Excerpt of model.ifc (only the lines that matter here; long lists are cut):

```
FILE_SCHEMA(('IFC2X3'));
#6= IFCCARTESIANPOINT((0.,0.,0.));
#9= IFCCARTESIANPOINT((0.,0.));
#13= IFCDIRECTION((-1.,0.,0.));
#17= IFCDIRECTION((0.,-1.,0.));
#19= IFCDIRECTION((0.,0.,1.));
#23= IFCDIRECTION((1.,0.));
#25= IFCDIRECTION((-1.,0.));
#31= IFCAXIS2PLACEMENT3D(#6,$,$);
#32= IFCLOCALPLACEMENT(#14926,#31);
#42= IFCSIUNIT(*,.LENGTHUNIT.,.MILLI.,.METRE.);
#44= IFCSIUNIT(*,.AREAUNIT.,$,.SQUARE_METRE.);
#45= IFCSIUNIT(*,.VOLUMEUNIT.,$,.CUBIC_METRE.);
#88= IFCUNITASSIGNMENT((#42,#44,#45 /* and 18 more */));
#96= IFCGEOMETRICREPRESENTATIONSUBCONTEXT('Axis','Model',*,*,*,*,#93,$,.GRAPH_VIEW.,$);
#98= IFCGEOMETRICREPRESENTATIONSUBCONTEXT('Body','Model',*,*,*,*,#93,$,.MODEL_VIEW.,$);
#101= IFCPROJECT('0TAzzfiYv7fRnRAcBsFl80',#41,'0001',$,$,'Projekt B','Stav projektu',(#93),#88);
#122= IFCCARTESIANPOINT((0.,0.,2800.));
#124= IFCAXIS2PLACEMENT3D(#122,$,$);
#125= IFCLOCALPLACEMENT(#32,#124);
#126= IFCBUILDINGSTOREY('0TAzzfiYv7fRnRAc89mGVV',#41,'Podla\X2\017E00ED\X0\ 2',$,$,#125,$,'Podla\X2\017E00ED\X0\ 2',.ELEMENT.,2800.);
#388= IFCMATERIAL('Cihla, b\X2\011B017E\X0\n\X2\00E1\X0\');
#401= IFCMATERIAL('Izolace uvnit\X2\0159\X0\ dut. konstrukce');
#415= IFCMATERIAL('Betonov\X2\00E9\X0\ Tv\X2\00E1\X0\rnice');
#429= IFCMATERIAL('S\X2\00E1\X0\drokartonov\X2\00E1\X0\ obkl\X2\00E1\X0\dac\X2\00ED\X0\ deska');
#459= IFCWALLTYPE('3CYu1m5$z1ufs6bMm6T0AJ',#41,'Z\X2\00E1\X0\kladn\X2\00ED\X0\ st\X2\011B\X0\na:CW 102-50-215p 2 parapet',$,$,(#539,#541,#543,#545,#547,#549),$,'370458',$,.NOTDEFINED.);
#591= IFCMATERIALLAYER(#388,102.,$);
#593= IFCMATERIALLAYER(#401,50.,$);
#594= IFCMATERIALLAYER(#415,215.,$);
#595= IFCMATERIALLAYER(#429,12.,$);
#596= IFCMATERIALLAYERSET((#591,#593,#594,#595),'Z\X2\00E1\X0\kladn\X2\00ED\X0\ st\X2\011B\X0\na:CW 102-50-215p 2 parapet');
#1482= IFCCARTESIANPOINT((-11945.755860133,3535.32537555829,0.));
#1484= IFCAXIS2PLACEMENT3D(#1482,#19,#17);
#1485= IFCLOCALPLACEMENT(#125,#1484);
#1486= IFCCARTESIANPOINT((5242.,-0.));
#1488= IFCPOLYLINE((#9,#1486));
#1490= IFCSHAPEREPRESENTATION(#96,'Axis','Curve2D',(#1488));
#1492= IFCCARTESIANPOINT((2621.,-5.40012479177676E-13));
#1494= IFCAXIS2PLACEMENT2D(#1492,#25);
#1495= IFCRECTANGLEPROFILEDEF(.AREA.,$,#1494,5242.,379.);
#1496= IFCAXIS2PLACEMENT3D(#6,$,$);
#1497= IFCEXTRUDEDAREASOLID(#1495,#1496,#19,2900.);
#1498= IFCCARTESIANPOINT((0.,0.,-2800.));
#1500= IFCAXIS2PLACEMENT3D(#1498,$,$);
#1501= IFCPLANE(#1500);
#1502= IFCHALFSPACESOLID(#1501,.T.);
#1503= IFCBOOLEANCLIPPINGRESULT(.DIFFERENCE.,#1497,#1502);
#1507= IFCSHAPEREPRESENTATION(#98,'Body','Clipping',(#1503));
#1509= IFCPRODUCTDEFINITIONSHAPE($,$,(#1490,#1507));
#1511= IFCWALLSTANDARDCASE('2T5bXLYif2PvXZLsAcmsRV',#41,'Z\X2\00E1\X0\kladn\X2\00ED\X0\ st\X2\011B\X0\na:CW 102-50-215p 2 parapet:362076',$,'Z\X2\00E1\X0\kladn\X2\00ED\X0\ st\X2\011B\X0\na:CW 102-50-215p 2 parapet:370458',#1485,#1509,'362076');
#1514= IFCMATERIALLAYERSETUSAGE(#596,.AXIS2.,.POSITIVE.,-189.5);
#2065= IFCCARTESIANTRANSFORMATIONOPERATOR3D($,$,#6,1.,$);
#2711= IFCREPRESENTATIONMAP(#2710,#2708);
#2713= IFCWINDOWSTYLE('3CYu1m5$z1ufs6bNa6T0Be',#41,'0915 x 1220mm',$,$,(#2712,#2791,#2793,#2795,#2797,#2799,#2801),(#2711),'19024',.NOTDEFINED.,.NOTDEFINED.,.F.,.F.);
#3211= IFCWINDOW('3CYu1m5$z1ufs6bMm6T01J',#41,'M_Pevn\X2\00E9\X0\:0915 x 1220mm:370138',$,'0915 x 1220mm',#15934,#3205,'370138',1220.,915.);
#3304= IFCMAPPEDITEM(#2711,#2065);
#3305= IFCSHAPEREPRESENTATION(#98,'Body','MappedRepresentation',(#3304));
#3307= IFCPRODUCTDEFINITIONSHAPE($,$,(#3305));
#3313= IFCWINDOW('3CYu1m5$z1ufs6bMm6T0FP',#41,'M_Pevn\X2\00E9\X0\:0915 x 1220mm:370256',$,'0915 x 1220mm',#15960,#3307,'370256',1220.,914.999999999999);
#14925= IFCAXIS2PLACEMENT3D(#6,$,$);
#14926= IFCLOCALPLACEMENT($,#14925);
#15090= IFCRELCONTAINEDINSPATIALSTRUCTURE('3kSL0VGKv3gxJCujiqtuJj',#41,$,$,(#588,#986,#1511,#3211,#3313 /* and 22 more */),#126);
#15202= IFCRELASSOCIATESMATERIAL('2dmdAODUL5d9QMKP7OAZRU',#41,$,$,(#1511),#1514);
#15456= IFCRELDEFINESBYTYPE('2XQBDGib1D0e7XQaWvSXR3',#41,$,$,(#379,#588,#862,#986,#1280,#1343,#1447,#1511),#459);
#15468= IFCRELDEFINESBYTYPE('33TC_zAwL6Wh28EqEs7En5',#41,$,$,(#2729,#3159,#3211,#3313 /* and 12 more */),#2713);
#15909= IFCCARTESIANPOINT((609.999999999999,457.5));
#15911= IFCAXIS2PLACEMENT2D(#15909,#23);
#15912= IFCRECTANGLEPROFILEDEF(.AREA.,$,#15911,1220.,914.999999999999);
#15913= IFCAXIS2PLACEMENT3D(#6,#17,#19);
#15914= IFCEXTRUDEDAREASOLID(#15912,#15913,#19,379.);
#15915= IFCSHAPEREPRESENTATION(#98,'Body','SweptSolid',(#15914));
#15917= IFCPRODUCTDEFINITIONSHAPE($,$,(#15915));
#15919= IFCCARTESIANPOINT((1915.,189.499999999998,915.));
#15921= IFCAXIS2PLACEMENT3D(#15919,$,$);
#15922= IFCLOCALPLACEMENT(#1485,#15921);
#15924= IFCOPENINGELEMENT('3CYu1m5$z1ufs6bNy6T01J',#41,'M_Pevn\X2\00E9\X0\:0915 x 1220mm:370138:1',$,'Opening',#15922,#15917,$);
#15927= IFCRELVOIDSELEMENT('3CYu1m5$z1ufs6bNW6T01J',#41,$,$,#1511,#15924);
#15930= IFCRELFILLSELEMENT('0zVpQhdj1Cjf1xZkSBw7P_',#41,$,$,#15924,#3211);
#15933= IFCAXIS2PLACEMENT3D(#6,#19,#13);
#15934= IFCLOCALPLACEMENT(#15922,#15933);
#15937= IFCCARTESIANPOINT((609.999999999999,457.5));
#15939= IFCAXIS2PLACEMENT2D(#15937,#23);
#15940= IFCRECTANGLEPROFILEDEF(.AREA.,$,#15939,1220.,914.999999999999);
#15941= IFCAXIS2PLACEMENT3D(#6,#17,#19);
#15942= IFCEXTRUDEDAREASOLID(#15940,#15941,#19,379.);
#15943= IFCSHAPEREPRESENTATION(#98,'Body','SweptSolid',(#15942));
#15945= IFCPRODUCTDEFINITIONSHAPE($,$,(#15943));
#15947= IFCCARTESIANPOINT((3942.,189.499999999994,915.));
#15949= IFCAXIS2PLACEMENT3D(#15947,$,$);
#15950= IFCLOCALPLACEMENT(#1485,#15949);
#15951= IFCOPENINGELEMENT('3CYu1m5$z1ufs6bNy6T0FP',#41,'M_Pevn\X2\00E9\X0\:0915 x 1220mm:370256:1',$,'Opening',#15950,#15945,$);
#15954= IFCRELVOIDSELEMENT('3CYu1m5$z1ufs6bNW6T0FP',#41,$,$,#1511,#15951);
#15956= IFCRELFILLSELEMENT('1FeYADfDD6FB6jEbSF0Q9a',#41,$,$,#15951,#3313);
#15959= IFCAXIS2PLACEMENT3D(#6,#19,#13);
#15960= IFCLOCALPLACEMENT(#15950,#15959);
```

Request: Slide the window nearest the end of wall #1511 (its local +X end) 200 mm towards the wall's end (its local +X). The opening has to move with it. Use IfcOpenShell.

```python
import ifcopenshell
import ifcopenshell.api.geometry
import ifcopenshell.util.placement

model = ifcopenshell.open("model.ifc")

window = model.by_id(3313)
opening = window.FillsVoids[0].RelatingOpeningElement
wall = opening.VoidsElements[0].RelatingBuildingElement

wall_matrix = ifcopenshell.util.placement.get_local_placement(wall.ObjectPlacement)
shift = wall_matrix[:3, 0] * 200.0
before = ifcopenshell.util.placement.get_local_placement(window.ObjectPlacement)[:3, 3].copy()

# The window is placed relative to its opening, so it follows when the opening moves.
matrix = ifcopenshell.util.placement.get_local_placement(opening.ObjectPlacement)
matrix[:3, 3] += shift
ifcopenshell.api.geometry.edit_object_placement(
    model, product=opening, matrix=matrix, is_si=False, should_transform_children=True
)

after = ifcopenshell.util.placement.get_local_placement(window.ObjectPlacement)[:3, 3]
print("window moved by", (after - before).round(3) + 0.0)

model.write("model-out.ifc")
```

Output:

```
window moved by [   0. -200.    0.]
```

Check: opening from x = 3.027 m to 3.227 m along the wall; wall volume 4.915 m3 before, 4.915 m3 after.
